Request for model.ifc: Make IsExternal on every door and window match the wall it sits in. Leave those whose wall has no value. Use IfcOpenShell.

First a look at what the model holds.

```python
import ifcopenshell
import ifcopenshell.util.element

model = ifcopenshell.open("model.ifc")
print(model.schema)
seen = {}
for e in model.by_type("IfcDoor") + model.by_type("IfcWindow"):
    if not e.FillsVoids:
        continue
    host = e.FillsVoids[0].RelatingOpeningElement.VoidsElements[0].RelatingBuildingElement
    own = ifcopenshell.util.element.get_pset(e, f"Pset_{e.is_a()[3:].removesuffix('StandardCase')}Common", "IsExternal")
    wall = ifcopenshell.util.element.get_pset(host, "Pset_WallCommon", "IsExternal")
    seen[e.is_a(), own, wall] = seen.get((e.is_a(), own, wall), 0) + 1
for (cls, own, wall), count in sorted(seen.items(), key=str):
    print(count, cls, "IsExternal:", own, "| host wall:", wall)
```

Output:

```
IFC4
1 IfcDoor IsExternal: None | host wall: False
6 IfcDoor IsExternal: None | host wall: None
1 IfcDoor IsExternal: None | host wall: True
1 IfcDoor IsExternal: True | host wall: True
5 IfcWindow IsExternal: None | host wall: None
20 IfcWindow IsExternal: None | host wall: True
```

```python
import ifcopenshell
import ifcopenshell.api.pset
import ifcopenshell.util.element

model = ifcopenshell.open("model.ifc")

count = 0
for ifc_class, pset_name in (("IfcDoor", "Pset_DoorCommon"), ("IfcWindow", "Pset_WindowCommon")):
    for e in model.by_type(ifc_class):
        if not e.FillsVoids:
            continue
        host = e.FillsVoids[0].RelatingOpeningElement.VoidsElements[0].RelatingBuildingElement
        external = ifcopenshell.util.element.get_pset(host, "Pset_WallCommon", "IsExternal")
        if external is None or ifcopenshell.util.element.get_pset(e, pset_name, "IsExternal") == external:
            continue
        pset = ifcopenshell.api.pset.add_pset(model, product=e, name=pset_name)
        ifcopenshell.api.pset.edit_pset(model, pset=pset, properties={"IsExternal": external})
        count += 1

print(count, "updated")

model.write("model-out.ifc")
```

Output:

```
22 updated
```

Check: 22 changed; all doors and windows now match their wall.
